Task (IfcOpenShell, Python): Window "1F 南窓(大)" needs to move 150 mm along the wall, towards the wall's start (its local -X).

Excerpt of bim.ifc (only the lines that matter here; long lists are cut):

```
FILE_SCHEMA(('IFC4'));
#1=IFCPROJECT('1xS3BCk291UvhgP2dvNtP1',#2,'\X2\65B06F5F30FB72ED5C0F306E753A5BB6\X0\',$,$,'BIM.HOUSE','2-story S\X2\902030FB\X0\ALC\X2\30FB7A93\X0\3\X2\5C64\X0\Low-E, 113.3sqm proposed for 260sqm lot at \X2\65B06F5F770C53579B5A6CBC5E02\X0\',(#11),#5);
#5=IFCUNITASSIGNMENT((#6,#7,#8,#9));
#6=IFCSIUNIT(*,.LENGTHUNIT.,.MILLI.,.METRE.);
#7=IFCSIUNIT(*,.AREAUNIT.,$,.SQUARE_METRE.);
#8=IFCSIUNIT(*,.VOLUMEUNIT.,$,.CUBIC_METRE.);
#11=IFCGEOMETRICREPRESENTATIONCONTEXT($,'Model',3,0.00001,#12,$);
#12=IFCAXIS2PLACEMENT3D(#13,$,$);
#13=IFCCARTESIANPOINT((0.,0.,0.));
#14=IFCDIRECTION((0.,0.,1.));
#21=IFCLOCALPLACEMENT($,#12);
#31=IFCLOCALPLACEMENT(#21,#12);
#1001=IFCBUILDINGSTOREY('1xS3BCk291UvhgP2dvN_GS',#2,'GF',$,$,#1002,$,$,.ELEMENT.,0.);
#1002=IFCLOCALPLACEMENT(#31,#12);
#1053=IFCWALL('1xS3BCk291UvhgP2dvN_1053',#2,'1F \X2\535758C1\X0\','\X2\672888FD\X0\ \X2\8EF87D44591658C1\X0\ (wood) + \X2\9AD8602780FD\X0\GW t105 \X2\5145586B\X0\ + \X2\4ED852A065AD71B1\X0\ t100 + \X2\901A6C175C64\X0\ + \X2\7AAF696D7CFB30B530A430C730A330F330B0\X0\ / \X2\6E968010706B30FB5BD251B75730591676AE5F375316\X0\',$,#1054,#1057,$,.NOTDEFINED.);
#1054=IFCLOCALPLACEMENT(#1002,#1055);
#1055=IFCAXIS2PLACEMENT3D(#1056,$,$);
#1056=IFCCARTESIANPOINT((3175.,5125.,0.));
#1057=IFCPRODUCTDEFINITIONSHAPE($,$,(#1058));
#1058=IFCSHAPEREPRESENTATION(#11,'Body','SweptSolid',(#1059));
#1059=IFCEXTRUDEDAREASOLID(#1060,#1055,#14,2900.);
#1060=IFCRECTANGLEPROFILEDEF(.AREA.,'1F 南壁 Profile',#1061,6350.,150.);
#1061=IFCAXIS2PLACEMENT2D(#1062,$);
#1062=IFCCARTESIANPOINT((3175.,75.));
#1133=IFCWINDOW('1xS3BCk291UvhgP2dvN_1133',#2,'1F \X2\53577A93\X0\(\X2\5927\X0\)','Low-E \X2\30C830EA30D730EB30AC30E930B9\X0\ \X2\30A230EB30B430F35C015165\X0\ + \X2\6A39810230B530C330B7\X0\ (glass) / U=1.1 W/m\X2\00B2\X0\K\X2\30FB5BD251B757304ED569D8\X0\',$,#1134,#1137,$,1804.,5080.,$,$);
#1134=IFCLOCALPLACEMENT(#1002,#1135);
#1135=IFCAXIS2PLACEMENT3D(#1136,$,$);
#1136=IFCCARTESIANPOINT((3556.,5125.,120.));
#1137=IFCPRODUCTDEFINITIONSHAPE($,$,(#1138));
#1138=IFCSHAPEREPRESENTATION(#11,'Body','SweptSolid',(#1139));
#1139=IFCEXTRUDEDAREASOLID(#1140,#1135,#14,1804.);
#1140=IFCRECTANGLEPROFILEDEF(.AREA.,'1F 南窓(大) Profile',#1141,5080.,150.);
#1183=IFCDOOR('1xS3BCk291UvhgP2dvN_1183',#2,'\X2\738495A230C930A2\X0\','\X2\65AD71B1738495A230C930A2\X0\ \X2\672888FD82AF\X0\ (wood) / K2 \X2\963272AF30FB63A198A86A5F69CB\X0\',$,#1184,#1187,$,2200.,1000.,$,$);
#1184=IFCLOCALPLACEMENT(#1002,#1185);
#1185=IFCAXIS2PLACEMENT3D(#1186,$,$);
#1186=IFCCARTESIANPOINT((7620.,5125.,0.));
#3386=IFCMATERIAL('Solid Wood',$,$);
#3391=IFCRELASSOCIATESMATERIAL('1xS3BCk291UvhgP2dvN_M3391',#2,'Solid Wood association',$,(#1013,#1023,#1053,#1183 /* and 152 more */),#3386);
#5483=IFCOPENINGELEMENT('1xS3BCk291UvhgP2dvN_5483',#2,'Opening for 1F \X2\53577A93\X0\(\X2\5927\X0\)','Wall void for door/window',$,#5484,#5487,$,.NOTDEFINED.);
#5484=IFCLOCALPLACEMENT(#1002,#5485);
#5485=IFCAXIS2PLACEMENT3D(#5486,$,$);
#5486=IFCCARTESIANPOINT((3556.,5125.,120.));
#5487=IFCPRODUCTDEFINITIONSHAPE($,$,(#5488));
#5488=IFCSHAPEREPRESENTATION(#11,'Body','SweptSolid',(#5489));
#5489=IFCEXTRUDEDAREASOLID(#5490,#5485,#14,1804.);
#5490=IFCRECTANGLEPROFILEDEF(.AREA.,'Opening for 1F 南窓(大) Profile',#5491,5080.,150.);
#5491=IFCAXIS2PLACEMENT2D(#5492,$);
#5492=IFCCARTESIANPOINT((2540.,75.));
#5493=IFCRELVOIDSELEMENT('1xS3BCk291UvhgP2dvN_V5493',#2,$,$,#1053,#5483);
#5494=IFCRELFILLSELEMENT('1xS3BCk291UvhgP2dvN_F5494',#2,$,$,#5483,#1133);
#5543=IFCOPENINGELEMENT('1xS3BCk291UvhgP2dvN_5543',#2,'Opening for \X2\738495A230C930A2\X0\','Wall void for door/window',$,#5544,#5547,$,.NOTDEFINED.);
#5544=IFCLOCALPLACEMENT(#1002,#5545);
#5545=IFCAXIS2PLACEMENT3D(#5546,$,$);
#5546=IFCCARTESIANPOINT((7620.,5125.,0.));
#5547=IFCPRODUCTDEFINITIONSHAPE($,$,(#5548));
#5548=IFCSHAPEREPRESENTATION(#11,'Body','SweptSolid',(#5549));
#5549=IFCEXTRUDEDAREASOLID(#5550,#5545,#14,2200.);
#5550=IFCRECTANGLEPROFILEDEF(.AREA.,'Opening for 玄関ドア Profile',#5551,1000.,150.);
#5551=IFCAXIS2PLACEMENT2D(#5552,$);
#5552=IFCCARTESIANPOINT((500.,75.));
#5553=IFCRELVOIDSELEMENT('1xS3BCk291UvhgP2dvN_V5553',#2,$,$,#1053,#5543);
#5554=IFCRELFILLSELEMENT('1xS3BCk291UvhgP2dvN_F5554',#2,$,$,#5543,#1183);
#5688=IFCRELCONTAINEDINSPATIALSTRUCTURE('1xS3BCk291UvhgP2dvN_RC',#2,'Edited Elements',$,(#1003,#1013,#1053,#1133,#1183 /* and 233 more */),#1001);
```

```python
import ifcopenshell
import ifcopenshell.api.geometry
import ifcopenshell.util.placement
import ifcopenshell.util.unit

model = ifcopenshell.open("bim.ifc")
unit_scale = ifcopenshell.util.unit.calculate_unit_scale(model)

window = model.by_guid("1xS3BCk291UvhgP2dvN_1133")
opening = window.FillsVoids[0].RelatingOpeningElement
wall = opening.VoidsElements[0].RelatingBuildingElement

wall_matrix = ifcopenshell.util.placement.get_local_placement(wall.ObjectPlacement)
shift = wall_matrix[:3, 0] * -0.15 / unit_scale
before = ifcopenshell.util.placement.get_local_placement(window.ObjectPlacement)[:3, 3].copy()

# The window is not placed relative to its opening, so move both.
for product in (opening, window):
    matrix = ifcopenshell.util.placement.get_local_placement(product.ObjectPlacement)
    matrix[:3, 3] += shift
    ifcopenshell.api.geometry.edit_object_placement(model, product=product, matrix=matrix, is_si=False)

after = ifcopenshell.util.placement.get_local_placement(window.ObjectPlacement)[:3, 3]
print("window moved by", (after - before).round(3) + 0.0)

model.write("bim_v2.ifc")
```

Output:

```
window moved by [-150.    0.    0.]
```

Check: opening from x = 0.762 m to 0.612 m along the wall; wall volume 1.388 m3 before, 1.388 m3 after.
